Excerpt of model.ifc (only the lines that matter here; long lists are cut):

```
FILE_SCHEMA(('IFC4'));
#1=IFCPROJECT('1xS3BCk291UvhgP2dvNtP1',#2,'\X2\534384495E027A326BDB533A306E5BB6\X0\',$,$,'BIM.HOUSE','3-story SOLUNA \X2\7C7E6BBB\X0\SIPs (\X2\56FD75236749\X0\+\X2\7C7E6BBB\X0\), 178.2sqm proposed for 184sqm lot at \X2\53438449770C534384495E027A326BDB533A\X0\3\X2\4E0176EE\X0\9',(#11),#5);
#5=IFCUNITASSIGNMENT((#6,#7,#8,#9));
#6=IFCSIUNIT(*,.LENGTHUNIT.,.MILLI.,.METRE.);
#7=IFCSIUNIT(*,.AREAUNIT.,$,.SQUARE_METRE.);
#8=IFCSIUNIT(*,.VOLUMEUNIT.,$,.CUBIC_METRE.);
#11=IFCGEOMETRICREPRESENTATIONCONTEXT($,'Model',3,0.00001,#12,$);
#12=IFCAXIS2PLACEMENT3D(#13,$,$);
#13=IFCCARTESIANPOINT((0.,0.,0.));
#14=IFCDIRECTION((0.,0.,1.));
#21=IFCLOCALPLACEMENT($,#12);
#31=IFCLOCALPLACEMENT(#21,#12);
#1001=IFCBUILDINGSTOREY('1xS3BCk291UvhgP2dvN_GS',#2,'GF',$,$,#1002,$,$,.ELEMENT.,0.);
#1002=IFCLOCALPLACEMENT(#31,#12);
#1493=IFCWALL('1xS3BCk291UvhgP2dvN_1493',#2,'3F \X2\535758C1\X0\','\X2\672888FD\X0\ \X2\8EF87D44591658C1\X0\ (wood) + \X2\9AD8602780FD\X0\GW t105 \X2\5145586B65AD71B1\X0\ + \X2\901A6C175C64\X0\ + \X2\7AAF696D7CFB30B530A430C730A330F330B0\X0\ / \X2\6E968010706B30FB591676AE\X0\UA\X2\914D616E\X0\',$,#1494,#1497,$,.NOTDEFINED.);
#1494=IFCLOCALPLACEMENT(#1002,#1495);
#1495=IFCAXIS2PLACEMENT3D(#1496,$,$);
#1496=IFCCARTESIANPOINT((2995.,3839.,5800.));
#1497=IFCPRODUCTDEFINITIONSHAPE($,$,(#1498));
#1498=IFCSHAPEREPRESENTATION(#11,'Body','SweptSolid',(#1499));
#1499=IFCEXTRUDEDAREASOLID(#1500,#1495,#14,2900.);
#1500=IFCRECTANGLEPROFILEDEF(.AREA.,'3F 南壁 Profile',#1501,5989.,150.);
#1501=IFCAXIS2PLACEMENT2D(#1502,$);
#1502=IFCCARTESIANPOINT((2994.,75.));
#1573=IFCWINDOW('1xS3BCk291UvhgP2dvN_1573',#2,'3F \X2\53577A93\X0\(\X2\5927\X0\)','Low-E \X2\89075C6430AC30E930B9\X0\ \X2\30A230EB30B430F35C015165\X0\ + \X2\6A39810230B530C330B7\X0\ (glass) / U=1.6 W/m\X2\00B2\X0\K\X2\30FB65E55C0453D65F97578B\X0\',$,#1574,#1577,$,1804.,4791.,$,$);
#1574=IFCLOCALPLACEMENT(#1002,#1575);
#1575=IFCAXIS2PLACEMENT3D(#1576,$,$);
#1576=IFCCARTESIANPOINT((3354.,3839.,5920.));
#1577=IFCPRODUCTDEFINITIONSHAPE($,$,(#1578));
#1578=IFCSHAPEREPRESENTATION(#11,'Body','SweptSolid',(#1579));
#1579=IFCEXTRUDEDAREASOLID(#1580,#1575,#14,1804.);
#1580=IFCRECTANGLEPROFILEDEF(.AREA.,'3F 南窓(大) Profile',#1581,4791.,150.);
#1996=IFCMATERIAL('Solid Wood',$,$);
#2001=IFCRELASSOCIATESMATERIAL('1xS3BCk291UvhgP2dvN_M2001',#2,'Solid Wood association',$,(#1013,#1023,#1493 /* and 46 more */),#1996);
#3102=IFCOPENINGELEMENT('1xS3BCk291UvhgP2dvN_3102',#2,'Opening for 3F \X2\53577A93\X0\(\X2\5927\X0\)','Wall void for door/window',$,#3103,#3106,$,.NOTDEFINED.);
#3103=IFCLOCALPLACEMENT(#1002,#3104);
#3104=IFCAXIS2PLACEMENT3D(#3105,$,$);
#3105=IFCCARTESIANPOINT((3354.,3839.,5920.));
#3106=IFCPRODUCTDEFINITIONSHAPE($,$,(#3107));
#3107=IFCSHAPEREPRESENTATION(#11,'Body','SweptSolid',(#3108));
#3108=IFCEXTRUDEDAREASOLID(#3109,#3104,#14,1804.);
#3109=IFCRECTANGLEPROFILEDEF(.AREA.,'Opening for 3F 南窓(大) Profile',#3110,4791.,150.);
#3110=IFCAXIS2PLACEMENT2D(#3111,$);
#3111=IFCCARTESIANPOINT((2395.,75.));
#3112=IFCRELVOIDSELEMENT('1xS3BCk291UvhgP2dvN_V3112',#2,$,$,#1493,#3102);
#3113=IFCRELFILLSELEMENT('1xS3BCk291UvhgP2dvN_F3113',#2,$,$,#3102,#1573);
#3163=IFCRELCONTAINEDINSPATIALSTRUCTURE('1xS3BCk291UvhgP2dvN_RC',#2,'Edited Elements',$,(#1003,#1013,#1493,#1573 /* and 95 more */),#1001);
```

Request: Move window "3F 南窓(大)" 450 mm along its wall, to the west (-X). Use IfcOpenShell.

```python
import ifcopenshell
import ifcopenshell.api.geometry
import ifcopenshell.util.placement
import ifcopenshell.util.unit

model = ifcopenshell.open("model.ifc")
unit_scale = ifcopenshell.util.unit.calculate_unit_scale(model)

window = model.by_guid("1xS3BCk291UvhgP2dvN_1573")
opening = window.FillsVoids[0].RelatingOpeningElement
wall = opening.VoidsElements[0].RelatingBuildingElement

wall_matrix = ifcopenshell.util.placement.get_local_placement(wall.ObjectPlacement)
shift = wall_matrix[:3, 0] * -0.45 / unit_scale
before = ifcopenshell.util.placement.get_local_placement(window.ObjectPlacement)[:3, 3].copy()

# The window is not placed relative to its opening, so move both.
for product in (opening, window):
    matrix = ifcopenshell.util.placement.get_local_placement(product.ObjectPlacement)
    matrix[:3, 3] += shift
    ifcopenshell.api.geometry.edit_object_placement(model, product=product, matrix=matrix, is_si=False)

after = ifcopenshell.util.placement.get_local_placement(window.ObjectPlacement)[:3, 3]
print("window moved by", (after - before).round(3) + 0.0)

model.write("model_rev.ifc")
```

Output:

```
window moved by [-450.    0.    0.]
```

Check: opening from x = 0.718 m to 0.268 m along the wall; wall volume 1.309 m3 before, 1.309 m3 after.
